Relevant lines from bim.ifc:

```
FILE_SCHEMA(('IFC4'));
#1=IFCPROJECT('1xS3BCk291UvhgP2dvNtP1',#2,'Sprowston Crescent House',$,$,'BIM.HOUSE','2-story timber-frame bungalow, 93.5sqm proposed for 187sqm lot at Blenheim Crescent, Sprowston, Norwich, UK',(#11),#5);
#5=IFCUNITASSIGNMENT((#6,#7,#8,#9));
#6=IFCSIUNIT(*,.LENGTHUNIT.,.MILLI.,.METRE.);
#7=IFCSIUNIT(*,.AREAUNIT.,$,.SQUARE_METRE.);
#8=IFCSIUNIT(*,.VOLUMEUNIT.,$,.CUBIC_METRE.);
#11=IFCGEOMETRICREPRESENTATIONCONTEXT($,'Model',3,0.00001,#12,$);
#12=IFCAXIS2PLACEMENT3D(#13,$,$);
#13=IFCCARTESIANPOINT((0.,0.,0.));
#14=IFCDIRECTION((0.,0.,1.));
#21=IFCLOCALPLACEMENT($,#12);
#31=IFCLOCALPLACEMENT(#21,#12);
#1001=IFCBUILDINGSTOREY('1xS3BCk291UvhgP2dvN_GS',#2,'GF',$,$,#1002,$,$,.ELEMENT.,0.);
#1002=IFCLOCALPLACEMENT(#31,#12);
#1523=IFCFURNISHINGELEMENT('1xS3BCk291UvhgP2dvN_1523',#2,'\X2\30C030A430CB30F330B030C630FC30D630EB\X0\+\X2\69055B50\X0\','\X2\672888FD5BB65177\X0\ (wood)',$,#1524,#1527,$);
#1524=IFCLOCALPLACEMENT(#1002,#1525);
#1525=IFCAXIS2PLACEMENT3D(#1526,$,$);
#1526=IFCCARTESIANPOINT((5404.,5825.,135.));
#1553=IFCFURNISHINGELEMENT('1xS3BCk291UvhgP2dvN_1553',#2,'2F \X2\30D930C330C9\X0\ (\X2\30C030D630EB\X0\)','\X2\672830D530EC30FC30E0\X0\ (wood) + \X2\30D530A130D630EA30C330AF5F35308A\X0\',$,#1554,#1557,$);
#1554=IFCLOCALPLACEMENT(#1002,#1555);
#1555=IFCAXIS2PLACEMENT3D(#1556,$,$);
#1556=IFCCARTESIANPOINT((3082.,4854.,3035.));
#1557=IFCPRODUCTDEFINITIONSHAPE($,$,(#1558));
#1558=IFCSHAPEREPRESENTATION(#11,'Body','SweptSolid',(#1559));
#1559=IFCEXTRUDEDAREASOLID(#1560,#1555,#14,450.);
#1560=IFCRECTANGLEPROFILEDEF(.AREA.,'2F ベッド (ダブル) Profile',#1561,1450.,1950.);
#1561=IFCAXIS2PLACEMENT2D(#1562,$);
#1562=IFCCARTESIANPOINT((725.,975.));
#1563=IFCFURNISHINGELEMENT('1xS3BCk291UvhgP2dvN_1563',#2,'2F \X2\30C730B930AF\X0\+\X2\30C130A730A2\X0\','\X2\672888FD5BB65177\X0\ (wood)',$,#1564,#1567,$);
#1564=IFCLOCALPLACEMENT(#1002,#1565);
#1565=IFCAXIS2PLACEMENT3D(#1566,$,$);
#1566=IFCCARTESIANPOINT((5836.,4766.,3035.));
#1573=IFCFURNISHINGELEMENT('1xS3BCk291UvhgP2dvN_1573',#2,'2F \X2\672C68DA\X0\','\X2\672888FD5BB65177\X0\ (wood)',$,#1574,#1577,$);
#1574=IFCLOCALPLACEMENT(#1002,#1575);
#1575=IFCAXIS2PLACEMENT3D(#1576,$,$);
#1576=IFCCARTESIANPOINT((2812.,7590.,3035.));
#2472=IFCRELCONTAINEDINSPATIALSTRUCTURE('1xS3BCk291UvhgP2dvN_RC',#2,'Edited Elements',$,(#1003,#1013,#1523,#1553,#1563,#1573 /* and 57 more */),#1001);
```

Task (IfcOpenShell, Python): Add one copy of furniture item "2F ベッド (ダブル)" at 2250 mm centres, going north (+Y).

```python
import numpy as np
import ifcopenshell
import ifcopenshell.api.geometry
import ifcopenshell.api.root
import ifcopenshell.util.element
import ifcopenshell.util.placement

model = ifcopenshell.open("bim.ifc")


def reuse_history(source, copy):
    """copy_class also copies each property set's owner history, people and application; keep the originals."""
    for rel in copy.IsDefinedBy:
        if rel.is_a("IfcRelDefinesByProperties") and (history := rel.RelatingPropertyDefinition.OwnerHistory):
            rel.RelatingPropertyDefinition.OwnerHistory = source.OwnerHistory
            ifcopenshell.util.element.remove_deep2(model, history)


source = model.by_guid("1xS3BCk291UvhgP2dvN_1553")
base = ifcopenshell.util.placement.get_local_placement(source.ObjectPlacement)
step = np.array([0.0, 1.0, 0.0]) * 2250.0

for i in range(1, 2):
    copy = ifcopenshell.api.root.copy_class(model, product=source)
    copy.Representation = ifcopenshell.util.element.copy_deep(
        model, source.Representation, exclude=["IfcGeometricRepresentationContext", "IfcRepresentationMap"]
    )
    reuse_history(source, copy)
    matrix = base.copy()
    matrix[:3, 3] += i * step
    print("added at", matrix[:3, 3].round(3) + 0.0)
    ifcopenshell.api.geometry.edit_object_placement(model, product=copy, matrix=matrix, is_si=False)

model.write("bim_updated.ifc")
```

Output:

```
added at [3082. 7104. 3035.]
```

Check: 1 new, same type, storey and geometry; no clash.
